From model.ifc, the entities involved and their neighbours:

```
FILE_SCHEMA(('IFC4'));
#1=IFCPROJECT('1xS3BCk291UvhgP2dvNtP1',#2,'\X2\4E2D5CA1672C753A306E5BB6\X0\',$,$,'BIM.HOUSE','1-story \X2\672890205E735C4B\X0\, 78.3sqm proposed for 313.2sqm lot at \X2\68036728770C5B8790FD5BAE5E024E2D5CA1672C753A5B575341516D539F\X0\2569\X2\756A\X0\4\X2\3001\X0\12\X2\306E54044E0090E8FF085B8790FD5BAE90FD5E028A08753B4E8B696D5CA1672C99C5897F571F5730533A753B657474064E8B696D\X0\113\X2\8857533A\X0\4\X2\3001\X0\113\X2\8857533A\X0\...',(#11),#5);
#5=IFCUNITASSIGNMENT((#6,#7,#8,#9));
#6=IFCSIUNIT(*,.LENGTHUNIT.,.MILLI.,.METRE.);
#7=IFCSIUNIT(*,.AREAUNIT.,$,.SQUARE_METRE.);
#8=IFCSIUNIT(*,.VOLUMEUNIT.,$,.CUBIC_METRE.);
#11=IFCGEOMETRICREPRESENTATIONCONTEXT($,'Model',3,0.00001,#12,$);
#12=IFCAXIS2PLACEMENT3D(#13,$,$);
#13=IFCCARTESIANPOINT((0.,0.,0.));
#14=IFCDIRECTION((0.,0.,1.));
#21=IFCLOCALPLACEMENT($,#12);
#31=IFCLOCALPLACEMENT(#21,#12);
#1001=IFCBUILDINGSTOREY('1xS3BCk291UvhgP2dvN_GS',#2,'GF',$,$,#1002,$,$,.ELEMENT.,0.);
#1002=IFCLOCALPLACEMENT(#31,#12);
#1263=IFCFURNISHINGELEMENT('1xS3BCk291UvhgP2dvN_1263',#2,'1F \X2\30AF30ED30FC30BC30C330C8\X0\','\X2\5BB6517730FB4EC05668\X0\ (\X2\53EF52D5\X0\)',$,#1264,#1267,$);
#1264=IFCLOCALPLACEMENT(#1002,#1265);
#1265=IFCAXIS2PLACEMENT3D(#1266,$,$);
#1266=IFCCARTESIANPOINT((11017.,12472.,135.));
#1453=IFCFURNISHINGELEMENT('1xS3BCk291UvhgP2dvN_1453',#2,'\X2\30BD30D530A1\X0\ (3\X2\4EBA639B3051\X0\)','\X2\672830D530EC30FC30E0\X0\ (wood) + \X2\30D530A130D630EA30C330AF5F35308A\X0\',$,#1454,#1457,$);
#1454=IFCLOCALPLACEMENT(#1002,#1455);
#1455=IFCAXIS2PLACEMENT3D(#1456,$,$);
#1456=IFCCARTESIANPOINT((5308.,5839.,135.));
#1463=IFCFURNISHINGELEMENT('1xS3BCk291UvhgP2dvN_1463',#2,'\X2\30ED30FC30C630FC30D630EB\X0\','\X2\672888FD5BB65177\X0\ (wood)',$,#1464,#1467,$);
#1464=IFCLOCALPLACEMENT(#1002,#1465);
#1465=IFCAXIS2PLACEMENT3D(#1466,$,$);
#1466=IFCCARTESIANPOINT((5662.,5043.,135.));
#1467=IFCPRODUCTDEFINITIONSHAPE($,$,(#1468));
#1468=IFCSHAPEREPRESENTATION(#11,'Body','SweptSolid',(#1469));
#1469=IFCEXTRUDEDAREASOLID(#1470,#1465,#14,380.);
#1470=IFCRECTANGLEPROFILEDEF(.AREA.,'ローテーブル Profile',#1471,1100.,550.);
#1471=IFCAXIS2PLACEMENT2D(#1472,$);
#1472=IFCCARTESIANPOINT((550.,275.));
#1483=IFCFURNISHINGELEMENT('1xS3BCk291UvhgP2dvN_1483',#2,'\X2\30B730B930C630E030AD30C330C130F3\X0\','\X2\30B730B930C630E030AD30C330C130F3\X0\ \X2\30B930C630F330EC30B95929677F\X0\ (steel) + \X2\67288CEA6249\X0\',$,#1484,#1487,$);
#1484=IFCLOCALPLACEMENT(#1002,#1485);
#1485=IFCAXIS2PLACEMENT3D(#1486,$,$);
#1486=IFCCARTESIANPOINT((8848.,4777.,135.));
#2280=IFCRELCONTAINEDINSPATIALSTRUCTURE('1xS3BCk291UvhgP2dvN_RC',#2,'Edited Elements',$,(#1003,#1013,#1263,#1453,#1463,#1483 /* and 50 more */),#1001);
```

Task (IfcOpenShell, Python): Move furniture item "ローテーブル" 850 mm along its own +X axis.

```python
import ifcopenshell
import ifcopenshell.api.geometry
import ifcopenshell.util.placement
import ifcopenshell.util.unit

model = ifcopenshell.open("model.ifc")
unit_scale = ifcopenshell.util.unit.calculate_unit_scale(model)

item = model.by_id(1463)
matrix = ifcopenshell.util.placement.get_local_placement(item.ObjectPlacement)
matrix[:3, 3] += matrix[:3, 0] * 0.85 / unit_scale
ifcopenshell.api.geometry.edit_object_placement(model, product=item, matrix=matrix, is_si=False)

print(ifcopenshell.util.placement.get_local_placement(item.ObjectPlacement).round(3) + 0.0)

model.write("model_v2.ifc")
```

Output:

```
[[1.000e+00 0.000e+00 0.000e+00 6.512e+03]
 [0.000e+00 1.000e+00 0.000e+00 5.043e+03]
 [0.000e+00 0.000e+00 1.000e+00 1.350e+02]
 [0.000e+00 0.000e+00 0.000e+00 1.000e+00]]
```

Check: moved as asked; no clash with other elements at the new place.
